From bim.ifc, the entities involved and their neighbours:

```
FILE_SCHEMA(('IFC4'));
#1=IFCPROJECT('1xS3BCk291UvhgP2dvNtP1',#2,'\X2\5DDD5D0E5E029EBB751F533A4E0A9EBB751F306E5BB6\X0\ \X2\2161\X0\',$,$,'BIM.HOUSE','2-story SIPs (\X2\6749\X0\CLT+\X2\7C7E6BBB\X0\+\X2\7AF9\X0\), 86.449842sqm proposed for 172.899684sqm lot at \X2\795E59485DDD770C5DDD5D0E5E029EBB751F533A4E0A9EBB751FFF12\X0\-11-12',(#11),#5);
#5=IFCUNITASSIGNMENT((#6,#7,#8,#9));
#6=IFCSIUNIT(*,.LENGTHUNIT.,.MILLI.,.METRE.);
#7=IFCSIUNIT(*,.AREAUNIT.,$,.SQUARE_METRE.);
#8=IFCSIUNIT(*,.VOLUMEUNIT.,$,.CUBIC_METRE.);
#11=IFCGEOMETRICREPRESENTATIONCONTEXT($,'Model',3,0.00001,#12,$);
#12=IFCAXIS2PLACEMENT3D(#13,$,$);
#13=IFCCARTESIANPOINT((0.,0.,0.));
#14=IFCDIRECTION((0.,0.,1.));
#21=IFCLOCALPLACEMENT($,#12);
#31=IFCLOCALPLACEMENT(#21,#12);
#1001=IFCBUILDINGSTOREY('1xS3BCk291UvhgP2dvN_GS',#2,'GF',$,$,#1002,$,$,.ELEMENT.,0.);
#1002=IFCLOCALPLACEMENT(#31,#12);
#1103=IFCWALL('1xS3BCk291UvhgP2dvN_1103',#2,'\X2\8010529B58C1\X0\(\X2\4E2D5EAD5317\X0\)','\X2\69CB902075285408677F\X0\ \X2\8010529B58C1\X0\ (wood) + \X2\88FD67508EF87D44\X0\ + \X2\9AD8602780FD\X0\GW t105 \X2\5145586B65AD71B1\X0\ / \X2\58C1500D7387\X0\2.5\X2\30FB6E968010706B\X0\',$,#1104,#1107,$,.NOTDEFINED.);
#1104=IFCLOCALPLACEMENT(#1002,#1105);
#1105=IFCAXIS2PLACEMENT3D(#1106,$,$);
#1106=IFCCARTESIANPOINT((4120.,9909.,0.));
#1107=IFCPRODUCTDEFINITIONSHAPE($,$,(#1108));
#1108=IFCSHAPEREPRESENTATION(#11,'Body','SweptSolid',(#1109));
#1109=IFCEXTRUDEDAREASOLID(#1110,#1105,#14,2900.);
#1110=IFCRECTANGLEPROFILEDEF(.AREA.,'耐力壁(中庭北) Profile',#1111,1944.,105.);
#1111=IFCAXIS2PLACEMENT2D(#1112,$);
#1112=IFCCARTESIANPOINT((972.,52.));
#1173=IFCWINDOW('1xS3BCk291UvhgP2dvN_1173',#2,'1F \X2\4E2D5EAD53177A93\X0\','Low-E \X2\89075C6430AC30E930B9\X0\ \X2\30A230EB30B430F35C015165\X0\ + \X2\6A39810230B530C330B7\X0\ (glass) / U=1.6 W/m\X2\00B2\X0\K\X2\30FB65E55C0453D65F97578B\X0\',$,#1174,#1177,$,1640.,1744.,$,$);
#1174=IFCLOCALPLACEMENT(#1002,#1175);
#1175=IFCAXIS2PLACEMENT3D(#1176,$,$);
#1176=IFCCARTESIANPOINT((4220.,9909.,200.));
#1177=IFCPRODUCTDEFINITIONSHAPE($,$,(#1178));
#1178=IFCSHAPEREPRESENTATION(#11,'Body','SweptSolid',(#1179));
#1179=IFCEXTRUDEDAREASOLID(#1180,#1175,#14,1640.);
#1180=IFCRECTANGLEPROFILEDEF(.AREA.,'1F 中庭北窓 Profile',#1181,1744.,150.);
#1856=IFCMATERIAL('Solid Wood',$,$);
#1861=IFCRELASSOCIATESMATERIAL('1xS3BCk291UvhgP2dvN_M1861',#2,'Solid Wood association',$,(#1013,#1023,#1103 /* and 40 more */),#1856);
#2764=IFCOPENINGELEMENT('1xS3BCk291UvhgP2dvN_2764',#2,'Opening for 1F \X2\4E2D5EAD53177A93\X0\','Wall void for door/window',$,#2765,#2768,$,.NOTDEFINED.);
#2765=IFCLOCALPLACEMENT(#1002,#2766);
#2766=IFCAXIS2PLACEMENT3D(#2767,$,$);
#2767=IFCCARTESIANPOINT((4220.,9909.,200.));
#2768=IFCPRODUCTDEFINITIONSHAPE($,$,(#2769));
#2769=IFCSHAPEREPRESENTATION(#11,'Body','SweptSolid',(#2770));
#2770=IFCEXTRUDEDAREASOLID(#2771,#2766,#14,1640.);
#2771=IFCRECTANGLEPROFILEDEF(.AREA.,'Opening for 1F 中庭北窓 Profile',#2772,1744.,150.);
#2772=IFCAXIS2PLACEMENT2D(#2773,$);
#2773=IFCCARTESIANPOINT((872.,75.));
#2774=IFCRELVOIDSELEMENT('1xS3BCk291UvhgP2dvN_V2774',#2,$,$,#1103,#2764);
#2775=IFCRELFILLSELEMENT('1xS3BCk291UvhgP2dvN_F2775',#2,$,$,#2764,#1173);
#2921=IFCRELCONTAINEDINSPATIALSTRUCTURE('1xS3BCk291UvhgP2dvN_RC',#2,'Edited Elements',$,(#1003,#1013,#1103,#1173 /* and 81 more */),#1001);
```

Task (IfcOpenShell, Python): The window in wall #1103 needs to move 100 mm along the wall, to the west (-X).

```python
import ifcopenshell
import ifcopenshell.api.geometry
import ifcopenshell.util.placement
import ifcopenshell.util.unit

model = ifcopenshell.open("bim.ifc")
unit_scale = ifcopenshell.util.unit.calculate_unit_scale(model)

window = model.by_id(1173)
opening = window.FillsVoids[0].RelatingOpeningElement
wall = opening.VoidsElements[0].RelatingBuildingElement

wall_matrix = ifcopenshell.util.placement.get_local_placement(wall.ObjectPlacement)
shift = wall_matrix[:3, 0] * -0.1 / unit_scale
before = ifcopenshell.util.placement.get_local_placement(window.ObjectPlacement)[:3, 3].copy()

# The window is not placed relative to its opening, so move both.
for product in (opening, window):
    matrix = ifcopenshell.util.placement.get_local_placement(product.ObjectPlacement)
    matrix[:3, 3] += shift
    ifcopenshell.api.geometry.edit_object_placement(model, product=product, matrix=matrix, is_si=False)

after = ifcopenshell.util.placement.get_local_placement(window.ObjectPlacement)[:3, 3]
print("window moved by", (after - before).round(3) + 0.0)

model.write("bim_v2.ifc")
```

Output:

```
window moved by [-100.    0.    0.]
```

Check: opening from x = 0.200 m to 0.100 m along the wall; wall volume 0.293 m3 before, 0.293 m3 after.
